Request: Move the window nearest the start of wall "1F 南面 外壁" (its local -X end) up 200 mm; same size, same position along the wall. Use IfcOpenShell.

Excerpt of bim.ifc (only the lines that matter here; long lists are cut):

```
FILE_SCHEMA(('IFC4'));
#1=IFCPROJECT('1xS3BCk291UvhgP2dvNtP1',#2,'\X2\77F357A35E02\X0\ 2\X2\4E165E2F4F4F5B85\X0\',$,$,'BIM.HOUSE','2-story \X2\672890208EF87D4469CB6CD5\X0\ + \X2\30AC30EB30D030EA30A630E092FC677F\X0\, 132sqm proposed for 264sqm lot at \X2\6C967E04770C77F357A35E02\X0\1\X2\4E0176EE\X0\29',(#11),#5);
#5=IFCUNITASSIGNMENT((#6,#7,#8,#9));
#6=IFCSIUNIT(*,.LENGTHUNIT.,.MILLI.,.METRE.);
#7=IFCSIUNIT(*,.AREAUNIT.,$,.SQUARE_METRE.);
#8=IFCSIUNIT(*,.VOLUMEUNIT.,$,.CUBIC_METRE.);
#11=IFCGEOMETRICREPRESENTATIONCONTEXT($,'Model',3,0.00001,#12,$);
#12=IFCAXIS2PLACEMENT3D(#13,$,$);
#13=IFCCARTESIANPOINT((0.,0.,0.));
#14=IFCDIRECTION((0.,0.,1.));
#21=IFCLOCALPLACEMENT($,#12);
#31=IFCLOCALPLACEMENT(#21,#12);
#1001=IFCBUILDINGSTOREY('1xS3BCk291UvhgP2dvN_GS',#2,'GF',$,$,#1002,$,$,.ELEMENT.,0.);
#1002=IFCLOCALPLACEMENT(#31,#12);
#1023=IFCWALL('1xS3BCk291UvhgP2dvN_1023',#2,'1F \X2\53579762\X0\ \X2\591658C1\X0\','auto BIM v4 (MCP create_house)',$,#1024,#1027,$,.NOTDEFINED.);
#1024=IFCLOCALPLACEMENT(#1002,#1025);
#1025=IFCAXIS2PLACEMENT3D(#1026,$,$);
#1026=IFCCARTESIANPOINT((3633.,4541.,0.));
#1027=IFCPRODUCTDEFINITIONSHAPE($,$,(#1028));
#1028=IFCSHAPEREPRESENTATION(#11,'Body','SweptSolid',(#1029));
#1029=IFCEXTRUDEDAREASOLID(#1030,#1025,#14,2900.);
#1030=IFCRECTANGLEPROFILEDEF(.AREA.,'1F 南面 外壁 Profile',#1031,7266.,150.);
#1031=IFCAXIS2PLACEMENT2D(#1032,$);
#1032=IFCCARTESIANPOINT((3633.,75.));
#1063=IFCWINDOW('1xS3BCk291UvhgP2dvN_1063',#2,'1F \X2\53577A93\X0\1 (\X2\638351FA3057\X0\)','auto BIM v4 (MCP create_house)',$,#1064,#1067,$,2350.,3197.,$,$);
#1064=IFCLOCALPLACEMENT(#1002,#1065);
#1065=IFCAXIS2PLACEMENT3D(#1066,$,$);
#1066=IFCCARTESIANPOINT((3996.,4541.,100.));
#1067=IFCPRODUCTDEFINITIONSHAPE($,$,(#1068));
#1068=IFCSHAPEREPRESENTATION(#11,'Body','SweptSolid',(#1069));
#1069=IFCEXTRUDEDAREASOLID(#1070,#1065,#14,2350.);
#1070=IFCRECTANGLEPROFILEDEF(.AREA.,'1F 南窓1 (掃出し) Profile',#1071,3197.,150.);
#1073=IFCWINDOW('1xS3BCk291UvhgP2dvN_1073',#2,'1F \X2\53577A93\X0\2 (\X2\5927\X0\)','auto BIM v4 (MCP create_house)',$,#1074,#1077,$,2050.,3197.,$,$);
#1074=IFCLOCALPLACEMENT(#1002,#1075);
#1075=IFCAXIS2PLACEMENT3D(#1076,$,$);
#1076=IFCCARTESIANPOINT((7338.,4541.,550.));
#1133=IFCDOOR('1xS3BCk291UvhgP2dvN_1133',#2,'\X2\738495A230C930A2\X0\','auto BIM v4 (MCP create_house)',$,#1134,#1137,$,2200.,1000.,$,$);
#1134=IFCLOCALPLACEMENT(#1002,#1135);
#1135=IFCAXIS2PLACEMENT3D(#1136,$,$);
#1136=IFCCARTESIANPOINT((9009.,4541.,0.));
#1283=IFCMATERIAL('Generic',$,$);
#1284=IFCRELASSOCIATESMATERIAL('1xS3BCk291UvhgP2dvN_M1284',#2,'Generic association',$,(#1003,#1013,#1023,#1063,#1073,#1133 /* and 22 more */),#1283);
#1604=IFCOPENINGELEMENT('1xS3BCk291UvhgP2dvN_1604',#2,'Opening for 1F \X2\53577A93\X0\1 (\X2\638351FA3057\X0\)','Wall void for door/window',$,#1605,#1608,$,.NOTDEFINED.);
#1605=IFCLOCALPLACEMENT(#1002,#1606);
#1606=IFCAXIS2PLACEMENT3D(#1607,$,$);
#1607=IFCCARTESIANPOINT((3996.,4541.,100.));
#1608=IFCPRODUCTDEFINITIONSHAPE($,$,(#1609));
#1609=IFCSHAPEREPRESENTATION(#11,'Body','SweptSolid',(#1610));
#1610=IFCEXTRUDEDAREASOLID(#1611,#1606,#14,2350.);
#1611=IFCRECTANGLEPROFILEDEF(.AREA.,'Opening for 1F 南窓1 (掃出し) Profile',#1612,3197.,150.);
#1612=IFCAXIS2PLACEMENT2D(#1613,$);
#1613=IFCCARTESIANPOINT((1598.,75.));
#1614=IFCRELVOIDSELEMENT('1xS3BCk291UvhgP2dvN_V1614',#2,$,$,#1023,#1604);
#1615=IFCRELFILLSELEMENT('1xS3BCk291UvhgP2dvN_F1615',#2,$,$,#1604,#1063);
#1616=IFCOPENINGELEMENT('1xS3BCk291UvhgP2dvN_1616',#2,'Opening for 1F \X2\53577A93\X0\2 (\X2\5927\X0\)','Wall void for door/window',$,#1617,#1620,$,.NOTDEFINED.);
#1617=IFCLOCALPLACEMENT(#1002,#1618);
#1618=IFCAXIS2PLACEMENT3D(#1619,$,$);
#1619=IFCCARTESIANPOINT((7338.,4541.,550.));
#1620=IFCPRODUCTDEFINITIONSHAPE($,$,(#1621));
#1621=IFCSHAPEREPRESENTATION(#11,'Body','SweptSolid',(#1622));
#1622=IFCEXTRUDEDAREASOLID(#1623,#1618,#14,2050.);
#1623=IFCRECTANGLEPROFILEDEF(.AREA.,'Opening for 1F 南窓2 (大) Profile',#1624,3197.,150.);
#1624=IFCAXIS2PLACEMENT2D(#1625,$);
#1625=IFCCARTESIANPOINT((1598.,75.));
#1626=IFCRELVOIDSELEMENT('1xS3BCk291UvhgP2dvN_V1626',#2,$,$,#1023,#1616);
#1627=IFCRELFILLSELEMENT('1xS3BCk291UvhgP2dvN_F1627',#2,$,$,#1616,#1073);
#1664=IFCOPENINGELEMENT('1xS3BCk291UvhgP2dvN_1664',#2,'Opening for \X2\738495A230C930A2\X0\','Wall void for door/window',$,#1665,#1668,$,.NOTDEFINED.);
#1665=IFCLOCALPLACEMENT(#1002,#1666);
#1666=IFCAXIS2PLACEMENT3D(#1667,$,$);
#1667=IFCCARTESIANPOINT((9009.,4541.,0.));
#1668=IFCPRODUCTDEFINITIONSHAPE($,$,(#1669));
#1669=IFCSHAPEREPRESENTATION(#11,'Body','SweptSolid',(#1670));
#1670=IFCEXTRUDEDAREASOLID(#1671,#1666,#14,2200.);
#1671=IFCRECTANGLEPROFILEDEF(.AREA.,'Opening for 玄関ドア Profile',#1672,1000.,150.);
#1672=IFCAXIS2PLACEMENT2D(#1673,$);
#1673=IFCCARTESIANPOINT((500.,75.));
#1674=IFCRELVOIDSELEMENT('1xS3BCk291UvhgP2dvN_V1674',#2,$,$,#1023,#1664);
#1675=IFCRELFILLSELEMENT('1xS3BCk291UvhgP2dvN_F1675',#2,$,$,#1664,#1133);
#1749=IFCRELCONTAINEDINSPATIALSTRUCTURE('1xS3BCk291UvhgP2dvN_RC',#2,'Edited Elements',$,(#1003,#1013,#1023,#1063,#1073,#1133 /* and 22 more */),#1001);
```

```python
import numpy as np
import ifcopenshell
import ifcopenshell.api.geometry
import ifcopenshell.util.placement
import ifcopenshell.util.unit

model = ifcopenshell.open("bim.ifc")
unit_scale = ifcopenshell.util.unit.calculate_unit_scale(model)

window = model.by_id(1063)
opening = window.FillsVoids[0].RelatingOpeningElement
dz = 200.0

shift = np.array([0.0, 0.0, dz])
# The window is not placed relative to its opening, so move both.
for product in (opening, window):
    matrix = ifcopenshell.util.placement.get_local_placement(product.ObjectPlacement)
    matrix[:3, 3] += shift
    ifcopenshell.api.geometry.edit_object_placement(model, product=product, matrix=matrix, is_si=False)

print(f"moved by {dz * unit_scale:+.3f} m")

model.write("bim_edited.ifc")
```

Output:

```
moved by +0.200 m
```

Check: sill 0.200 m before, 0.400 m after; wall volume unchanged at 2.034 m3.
